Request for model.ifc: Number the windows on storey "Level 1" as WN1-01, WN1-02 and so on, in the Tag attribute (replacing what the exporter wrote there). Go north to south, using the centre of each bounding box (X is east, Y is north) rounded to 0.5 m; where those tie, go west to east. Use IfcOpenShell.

First a look at what the model holds.

```python
import ifcopenshell
import ifcopenshell.util.element
import ifcopenshell.util.placement

model = ifcopenshell.open("model.ifc")
print(model.schema)
storey = next(s for s in model.by_type("IfcBuildingStorey") if s.Name == "Level 1")
windows = [e for e in ifcopenshell.util.element.get_decomposition(storey) if e.is_a("IfcWindow")]
for e in sorted(windows, key=lambda e: e.id()):
    origin = ifcopenshell.util.placement.get_local_placement(e.ObjectPlacement)[:3, 3]
    print(e.id(), e.Tag, e.Name, origin.round(2) + 0.0, sep=" | ")
```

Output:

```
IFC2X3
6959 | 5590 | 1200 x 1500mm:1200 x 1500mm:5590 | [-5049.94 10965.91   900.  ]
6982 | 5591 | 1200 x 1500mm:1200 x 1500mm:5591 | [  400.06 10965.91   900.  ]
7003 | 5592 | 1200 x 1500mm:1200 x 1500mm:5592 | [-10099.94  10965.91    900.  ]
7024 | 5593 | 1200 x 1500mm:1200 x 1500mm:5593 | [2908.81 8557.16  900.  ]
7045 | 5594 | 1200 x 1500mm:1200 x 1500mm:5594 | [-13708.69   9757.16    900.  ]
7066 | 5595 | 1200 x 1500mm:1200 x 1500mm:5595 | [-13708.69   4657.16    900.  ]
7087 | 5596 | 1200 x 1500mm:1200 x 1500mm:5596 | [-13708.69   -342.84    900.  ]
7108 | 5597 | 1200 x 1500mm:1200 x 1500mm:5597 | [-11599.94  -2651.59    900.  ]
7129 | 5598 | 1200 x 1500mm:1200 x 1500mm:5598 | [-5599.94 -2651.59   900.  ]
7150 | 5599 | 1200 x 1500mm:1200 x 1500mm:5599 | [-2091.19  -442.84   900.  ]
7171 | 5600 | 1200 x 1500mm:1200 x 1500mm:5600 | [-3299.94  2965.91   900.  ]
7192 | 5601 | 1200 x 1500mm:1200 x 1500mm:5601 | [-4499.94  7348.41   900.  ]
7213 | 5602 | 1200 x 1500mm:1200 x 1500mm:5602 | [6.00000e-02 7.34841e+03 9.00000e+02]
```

```python
import ifcopenshell
import ifcopenshell.geom
import ifcopenshell.util.element
import ifcopenshell.util.shape

model = ifcopenshell.open("model.ifc")
settings = ifcopenshell.geom.settings()
settings.set("use-world-coords", True)


def centre(element):
    shape = ifcopenshell.geom.create_shape(settings, element)
    return ifcopenshell.util.shape.get_bbox_centroid(shape.geometry)


storey = next(s for s in model.by_type("IfcBuildingStorey") if s.Name == "Level 1")
windows = [e for e in ifcopenshell.util.element.get_decomposition(storey) if e.is_a("IfcWindow")]

# Insertion points can sit at a corner or the storey origin, so sort by the geometry (in metres).
centres = {e: centre(e) for e in windows}
windows.sort(key=lambda e: (-round(centres[e][1] / 0.5), centres[e][0]))

for i, e in enumerate(windows, start=1):
    number = f"WN1-{i:02d}"
    e.Tag = number
    print(e.id(), number)

model.write("model_rev.ifc")
```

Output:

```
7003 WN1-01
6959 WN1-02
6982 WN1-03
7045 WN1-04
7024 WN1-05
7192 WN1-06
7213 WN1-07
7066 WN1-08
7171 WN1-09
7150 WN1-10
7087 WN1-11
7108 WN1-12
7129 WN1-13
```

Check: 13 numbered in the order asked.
